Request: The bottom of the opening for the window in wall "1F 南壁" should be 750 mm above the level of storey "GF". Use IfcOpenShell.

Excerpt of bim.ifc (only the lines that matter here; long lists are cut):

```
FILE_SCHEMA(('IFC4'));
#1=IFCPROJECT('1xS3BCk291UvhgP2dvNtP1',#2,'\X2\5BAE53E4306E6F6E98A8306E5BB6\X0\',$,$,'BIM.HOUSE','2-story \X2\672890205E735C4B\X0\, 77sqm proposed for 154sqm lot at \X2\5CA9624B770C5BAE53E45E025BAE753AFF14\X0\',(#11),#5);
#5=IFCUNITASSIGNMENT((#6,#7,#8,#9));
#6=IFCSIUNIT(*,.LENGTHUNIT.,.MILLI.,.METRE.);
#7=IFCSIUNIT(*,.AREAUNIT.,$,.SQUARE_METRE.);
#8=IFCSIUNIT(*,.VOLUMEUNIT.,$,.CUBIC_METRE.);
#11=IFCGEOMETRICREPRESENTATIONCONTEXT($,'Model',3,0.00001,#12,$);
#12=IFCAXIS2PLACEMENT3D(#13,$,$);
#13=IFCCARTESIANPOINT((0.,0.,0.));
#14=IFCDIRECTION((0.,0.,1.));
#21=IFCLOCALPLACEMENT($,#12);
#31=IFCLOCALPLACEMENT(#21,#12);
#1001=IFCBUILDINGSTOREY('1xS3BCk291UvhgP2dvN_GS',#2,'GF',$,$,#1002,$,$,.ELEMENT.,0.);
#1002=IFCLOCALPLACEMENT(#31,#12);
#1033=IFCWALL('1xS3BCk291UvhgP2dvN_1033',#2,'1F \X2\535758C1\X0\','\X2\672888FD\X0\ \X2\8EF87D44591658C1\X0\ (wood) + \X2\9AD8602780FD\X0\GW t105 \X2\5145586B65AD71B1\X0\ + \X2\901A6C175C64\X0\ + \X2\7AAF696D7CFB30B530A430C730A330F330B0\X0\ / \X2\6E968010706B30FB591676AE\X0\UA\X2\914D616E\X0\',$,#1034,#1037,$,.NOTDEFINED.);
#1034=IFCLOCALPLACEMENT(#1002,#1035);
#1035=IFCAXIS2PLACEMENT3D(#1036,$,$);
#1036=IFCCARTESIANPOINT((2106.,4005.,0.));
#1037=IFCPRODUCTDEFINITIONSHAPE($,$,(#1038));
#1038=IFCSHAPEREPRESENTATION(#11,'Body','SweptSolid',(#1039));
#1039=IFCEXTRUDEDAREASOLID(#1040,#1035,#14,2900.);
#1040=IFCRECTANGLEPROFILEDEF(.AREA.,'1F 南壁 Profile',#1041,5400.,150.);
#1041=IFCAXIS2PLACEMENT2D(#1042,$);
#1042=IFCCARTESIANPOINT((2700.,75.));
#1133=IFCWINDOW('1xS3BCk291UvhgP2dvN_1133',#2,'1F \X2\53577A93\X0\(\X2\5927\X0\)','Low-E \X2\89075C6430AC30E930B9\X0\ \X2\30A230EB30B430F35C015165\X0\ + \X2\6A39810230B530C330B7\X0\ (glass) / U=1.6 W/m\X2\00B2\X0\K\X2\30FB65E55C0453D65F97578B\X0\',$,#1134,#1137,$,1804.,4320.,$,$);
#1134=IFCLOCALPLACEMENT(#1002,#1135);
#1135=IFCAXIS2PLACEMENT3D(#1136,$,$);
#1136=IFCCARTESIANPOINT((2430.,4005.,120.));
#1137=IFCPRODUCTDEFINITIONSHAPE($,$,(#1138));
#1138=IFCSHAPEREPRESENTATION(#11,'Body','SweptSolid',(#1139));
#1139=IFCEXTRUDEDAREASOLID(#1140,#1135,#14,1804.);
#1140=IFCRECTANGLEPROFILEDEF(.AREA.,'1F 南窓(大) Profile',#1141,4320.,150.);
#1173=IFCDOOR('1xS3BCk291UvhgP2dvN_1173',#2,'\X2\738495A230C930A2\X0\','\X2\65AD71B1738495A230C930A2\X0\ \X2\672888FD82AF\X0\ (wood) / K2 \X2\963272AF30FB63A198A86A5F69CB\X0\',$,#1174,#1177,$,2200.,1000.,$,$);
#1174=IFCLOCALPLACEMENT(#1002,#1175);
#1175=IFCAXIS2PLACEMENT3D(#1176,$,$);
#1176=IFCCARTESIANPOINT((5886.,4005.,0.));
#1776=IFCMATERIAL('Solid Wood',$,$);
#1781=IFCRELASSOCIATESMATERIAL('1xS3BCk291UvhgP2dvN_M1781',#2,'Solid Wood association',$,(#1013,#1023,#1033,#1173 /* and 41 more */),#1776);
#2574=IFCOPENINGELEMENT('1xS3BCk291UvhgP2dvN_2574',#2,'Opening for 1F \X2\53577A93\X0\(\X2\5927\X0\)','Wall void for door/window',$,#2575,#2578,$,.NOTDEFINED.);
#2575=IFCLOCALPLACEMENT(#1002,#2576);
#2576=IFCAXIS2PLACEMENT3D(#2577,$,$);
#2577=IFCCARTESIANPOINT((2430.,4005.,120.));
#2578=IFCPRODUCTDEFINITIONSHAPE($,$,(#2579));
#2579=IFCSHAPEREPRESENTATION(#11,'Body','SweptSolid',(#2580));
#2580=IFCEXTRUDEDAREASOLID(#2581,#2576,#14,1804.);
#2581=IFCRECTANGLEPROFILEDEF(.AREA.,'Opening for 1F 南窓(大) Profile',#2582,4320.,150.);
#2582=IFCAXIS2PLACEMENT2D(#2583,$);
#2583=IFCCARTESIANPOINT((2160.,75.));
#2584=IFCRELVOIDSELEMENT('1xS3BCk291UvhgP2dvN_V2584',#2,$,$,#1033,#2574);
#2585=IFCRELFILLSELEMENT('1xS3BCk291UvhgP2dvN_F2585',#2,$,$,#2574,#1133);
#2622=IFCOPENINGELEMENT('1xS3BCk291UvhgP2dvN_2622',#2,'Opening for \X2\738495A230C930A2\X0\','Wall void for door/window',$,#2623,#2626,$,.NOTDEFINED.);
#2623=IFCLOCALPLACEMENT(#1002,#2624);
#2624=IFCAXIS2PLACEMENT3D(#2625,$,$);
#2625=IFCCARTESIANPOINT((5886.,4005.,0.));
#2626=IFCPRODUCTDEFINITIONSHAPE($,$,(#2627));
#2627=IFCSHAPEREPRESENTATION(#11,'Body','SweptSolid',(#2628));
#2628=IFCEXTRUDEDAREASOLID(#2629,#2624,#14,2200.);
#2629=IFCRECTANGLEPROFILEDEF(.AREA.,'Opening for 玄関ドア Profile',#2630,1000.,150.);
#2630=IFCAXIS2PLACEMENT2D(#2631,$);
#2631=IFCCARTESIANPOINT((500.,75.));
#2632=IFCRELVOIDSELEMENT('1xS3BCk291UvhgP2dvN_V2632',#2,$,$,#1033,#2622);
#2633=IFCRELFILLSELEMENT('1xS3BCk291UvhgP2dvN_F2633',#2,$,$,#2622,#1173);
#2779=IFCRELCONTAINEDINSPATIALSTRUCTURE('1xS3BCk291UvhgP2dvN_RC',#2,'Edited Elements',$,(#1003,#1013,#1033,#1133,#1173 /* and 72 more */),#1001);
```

```python
import numpy as np
import ifcopenshell
import ifcopenshell.api.geometry
import ifcopenshell.geom
import ifcopenshell.util.element
import ifcopenshell.util.placement
import ifcopenshell.util.shape
import ifcopenshell.util.unit

model = ifcopenshell.open("bim.ifc")
unit_scale = ifcopenshell.util.unit.calculate_unit_scale(model)

window = model.by_id(1133)
opening = window.FillsVoids[0].RelatingOpeningElement
storey = ifcopenshell.util.element.get_container(window, ifc_class="IfcBuildingStorey")
level = ifcopenshell.util.placement.get_local_placement(storey.ObjectPlacement)[2, 3]

# The opening's origin need not be at the sill, so measure its lowest point.
shape = ifcopenshell.geom.create_shape(ifcopenshell.geom.settings(), opening)
bottom = ifcopenshell.util.shape.get_shape_bottom_elevation(shape, shape.geometry) / unit_scale
dz = level + 750.0 - bottom

shift = np.array([0.0, 0.0, dz])
# The window is not placed relative to its opening, so move both.
for product in (opening, window):
    matrix = ifcopenshell.util.placement.get_local_placement(product.ObjectPlacement)
    matrix[:3, 3] += shift
    ifcopenshell.api.geometry.edit_object_placement(model, product=product, matrix=matrix, is_si=False)

print(f"moved by {dz * unit_scale:+.3f} m")

model.write("bim_edited.ifc")
```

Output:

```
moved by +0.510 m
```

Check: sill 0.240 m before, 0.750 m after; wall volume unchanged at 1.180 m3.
